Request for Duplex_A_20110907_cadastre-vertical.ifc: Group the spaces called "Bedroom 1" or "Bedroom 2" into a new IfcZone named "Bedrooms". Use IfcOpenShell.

First a look at what the model holds.

```python
import ifcopenshell

model = ifcopenshell.open("Duplex_A_20110907_cadastre-vertical.ifc")
print(model.schema)
seen = {}
for space in model.by_type("IfcSpace"):
    seen[space.LongName] = seen.get(space.LongName, 0) + 1
for name, count in sorted(seen.items(), key=str):
    print(count, "x", name)
print("zones:", [z.Name for z in model.by_type("IfcZone")][:20])
```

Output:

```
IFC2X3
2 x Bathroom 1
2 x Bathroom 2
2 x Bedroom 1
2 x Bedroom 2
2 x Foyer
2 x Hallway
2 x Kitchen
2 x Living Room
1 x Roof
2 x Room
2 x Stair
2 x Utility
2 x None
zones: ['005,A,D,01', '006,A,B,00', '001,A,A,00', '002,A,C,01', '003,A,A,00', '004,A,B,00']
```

```python
import ifcopenshell
import ifcopenshell.api.group
import ifcopenshell.api.root

model = ifcopenshell.open("Duplex_A_20110907_cadastre-vertical.ifc")

names = {"Bedroom 1", "Bedroom 2"}
spaces = [s for s in model.by_type("IfcSpace") if s.LongName in names]

zone = ifcopenshell.api.root.create_entity(model, ifc_class="IfcZone", name="Bedrooms")
ifcopenshell.api.group.assign_group(model, products=spaces, group=zone)
print(len(spaces), "spaces in", zone.Name)

model.write("Duplex_A_20110907_cadastre-vertical-out.ifc")
```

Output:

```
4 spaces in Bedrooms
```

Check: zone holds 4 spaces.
